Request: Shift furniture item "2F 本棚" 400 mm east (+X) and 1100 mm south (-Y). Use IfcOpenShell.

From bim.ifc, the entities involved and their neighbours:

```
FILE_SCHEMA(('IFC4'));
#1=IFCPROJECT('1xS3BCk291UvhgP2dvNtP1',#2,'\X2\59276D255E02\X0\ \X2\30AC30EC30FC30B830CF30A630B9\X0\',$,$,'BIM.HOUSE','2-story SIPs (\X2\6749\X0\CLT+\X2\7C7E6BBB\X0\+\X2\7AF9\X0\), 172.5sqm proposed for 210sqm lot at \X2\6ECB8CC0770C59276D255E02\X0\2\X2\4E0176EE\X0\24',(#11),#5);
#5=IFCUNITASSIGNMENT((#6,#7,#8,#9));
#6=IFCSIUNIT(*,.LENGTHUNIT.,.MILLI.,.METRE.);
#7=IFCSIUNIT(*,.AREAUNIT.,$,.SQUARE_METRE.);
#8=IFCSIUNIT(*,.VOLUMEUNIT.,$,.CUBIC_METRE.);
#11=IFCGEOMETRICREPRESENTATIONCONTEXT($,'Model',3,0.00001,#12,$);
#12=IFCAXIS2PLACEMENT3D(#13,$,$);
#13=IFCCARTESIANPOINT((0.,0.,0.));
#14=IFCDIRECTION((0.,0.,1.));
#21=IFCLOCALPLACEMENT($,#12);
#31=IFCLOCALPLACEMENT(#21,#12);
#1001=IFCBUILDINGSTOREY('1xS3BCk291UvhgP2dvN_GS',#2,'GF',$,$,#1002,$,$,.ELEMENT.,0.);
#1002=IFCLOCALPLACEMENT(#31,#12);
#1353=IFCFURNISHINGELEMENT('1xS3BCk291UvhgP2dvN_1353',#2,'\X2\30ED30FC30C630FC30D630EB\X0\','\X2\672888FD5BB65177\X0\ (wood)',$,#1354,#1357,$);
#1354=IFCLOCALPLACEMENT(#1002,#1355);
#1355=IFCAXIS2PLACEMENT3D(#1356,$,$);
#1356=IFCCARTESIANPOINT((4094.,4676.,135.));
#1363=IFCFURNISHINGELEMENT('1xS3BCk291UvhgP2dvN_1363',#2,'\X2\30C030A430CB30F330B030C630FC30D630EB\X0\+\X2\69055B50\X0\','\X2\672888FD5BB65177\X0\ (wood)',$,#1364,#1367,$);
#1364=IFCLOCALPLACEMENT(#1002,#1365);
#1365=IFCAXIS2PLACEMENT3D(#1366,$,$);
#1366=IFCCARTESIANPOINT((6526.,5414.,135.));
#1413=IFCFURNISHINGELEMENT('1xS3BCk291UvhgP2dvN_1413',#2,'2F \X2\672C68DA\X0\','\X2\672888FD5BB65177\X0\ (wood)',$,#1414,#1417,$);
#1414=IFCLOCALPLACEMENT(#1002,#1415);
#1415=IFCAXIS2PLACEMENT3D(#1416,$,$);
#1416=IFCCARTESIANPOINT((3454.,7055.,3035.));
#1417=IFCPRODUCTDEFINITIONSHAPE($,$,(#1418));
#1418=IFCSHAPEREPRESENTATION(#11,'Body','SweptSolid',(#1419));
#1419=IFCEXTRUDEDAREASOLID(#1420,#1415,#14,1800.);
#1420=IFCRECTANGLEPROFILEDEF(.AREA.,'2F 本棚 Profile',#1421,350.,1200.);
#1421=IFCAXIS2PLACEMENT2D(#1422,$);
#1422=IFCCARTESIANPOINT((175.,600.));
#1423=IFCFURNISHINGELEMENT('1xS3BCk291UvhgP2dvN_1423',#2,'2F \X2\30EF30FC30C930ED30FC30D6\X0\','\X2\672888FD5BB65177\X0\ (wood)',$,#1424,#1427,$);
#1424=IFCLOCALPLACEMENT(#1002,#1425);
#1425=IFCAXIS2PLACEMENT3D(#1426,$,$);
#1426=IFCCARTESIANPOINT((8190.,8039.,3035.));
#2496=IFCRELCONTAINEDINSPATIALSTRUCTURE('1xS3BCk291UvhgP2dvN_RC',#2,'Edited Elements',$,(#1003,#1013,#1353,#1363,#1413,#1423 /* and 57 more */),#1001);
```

```python
import ifcopenshell
import ifcopenshell.api.geometry
import ifcopenshell.util.placement
import ifcopenshell.util.unit

model = ifcopenshell.open("bim.ifc")
unit_scale = ifcopenshell.util.unit.calculate_unit_scale(model)

item = model.by_id(1413)
matrix = ifcopenshell.util.placement.get_local_placement(item.ObjectPlacement)
matrix[0, 3] += 0.4 / unit_scale
matrix[1, 3] -= 1.1 / unit_scale
ifcopenshell.api.geometry.edit_object_placement(model, product=item, matrix=matrix, is_si=False)

print(ifcopenshell.util.placement.get_local_placement(item.ObjectPlacement).round(3) + 0.0)

model.write("bim_v2.ifc")
```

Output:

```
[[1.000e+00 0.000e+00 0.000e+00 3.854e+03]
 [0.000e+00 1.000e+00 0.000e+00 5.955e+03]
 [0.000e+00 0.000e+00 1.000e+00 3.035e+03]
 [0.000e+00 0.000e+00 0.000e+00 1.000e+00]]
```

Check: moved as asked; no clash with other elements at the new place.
